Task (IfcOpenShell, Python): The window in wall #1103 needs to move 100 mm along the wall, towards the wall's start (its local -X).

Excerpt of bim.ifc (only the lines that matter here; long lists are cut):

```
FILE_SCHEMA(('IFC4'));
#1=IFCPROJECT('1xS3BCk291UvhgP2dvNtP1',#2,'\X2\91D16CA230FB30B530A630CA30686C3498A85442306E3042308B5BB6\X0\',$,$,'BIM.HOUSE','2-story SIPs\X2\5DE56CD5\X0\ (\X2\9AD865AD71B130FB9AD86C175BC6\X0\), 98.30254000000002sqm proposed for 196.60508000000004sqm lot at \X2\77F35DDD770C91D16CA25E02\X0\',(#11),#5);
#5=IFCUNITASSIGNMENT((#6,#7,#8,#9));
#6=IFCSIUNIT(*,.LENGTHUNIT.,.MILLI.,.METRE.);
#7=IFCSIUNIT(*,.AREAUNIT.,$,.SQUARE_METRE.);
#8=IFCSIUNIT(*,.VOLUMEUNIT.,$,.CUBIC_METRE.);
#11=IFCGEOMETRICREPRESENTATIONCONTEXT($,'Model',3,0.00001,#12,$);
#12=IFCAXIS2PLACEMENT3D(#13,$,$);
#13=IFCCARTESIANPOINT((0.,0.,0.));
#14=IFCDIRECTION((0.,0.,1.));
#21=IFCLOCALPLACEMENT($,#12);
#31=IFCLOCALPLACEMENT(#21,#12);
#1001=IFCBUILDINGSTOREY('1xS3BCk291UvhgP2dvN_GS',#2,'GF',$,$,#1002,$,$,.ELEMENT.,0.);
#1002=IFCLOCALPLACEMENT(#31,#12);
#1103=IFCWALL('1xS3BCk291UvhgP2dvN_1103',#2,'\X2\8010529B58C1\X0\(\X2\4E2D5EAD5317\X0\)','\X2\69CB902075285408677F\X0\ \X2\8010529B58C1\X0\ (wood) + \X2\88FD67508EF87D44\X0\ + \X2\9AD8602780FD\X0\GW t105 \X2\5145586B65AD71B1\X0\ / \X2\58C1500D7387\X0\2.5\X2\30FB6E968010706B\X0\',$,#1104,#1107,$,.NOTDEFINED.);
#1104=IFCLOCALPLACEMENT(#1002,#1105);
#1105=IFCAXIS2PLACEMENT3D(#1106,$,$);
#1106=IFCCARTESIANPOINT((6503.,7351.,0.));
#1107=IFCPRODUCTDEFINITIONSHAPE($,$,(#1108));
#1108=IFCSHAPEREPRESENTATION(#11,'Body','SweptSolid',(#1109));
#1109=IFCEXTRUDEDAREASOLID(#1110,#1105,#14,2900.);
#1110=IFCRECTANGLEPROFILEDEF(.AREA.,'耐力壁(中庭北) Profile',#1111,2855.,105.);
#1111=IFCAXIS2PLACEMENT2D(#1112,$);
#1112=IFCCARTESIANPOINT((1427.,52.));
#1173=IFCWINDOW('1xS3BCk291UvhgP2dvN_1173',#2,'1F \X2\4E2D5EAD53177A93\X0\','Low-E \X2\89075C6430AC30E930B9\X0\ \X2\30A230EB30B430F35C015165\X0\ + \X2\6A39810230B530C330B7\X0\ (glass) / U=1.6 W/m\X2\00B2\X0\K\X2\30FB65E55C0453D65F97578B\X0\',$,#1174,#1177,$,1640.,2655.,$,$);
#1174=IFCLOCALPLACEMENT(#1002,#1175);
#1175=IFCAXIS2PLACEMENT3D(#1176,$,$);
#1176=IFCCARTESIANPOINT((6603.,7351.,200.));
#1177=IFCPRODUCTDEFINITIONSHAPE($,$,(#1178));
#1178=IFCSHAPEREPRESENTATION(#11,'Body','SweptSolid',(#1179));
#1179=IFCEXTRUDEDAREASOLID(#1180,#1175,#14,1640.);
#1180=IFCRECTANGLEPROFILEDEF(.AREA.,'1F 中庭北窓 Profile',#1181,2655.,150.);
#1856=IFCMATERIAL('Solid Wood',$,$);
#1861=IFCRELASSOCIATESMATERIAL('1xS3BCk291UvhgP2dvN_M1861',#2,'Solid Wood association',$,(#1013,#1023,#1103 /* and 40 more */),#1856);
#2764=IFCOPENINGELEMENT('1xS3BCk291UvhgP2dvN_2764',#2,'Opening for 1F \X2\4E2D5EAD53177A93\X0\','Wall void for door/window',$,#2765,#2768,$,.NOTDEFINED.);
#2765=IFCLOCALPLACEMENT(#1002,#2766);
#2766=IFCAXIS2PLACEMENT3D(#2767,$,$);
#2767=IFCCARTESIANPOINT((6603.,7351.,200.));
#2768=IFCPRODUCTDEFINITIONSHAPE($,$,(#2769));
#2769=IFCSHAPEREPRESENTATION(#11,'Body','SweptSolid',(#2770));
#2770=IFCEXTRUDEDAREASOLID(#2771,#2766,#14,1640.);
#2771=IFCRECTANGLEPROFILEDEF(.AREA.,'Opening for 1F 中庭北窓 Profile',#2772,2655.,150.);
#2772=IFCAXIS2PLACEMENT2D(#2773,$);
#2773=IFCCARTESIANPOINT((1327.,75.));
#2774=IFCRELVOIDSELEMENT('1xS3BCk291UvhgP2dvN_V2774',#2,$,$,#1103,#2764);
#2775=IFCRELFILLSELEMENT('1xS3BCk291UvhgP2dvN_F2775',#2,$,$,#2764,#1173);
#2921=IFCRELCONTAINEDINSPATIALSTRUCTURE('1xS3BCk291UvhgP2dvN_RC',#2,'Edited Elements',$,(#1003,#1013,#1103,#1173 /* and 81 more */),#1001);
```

```python
import ifcopenshell
import ifcopenshell.api.geometry
import ifcopenshell.util.placement
import ifcopenshell.util.unit

model = ifcopenshell.open("bim.ifc")
unit_scale = ifcopenshell.util.unit.calculate_unit_scale(model)

window = model.by_id(1173)
opening = window.FillsVoids[0].RelatingOpeningElement
wall = opening.VoidsElements[0].RelatingBuildingElement

wall_matrix = ifcopenshell.util.placement.get_local_placement(wall.ObjectPlacement)
shift = wall_matrix[:3, 0] * -0.1 / unit_scale
before = ifcopenshell.util.placement.get_local_placement(window.ObjectPlacement)[:3, 3].copy()

# The window is not placed relative to its opening, so move both.
for product in (opening, window):
    matrix = ifcopenshell.util.placement.get_local_placement(product.ObjectPlacement)
    matrix[:3, 3] += shift
    ifcopenshell.api.geometry.edit_object_placement(model, product=product, matrix=matrix, is_si=False)

after = ifcopenshell.util.placement.get_local_placement(window.ObjectPlacement)[:3, 3]
print("window moved by", (after - before).round(3) + 0.0)

model.write("bim_rev.ifc")
```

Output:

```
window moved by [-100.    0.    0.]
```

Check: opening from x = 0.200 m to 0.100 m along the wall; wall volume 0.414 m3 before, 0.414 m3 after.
